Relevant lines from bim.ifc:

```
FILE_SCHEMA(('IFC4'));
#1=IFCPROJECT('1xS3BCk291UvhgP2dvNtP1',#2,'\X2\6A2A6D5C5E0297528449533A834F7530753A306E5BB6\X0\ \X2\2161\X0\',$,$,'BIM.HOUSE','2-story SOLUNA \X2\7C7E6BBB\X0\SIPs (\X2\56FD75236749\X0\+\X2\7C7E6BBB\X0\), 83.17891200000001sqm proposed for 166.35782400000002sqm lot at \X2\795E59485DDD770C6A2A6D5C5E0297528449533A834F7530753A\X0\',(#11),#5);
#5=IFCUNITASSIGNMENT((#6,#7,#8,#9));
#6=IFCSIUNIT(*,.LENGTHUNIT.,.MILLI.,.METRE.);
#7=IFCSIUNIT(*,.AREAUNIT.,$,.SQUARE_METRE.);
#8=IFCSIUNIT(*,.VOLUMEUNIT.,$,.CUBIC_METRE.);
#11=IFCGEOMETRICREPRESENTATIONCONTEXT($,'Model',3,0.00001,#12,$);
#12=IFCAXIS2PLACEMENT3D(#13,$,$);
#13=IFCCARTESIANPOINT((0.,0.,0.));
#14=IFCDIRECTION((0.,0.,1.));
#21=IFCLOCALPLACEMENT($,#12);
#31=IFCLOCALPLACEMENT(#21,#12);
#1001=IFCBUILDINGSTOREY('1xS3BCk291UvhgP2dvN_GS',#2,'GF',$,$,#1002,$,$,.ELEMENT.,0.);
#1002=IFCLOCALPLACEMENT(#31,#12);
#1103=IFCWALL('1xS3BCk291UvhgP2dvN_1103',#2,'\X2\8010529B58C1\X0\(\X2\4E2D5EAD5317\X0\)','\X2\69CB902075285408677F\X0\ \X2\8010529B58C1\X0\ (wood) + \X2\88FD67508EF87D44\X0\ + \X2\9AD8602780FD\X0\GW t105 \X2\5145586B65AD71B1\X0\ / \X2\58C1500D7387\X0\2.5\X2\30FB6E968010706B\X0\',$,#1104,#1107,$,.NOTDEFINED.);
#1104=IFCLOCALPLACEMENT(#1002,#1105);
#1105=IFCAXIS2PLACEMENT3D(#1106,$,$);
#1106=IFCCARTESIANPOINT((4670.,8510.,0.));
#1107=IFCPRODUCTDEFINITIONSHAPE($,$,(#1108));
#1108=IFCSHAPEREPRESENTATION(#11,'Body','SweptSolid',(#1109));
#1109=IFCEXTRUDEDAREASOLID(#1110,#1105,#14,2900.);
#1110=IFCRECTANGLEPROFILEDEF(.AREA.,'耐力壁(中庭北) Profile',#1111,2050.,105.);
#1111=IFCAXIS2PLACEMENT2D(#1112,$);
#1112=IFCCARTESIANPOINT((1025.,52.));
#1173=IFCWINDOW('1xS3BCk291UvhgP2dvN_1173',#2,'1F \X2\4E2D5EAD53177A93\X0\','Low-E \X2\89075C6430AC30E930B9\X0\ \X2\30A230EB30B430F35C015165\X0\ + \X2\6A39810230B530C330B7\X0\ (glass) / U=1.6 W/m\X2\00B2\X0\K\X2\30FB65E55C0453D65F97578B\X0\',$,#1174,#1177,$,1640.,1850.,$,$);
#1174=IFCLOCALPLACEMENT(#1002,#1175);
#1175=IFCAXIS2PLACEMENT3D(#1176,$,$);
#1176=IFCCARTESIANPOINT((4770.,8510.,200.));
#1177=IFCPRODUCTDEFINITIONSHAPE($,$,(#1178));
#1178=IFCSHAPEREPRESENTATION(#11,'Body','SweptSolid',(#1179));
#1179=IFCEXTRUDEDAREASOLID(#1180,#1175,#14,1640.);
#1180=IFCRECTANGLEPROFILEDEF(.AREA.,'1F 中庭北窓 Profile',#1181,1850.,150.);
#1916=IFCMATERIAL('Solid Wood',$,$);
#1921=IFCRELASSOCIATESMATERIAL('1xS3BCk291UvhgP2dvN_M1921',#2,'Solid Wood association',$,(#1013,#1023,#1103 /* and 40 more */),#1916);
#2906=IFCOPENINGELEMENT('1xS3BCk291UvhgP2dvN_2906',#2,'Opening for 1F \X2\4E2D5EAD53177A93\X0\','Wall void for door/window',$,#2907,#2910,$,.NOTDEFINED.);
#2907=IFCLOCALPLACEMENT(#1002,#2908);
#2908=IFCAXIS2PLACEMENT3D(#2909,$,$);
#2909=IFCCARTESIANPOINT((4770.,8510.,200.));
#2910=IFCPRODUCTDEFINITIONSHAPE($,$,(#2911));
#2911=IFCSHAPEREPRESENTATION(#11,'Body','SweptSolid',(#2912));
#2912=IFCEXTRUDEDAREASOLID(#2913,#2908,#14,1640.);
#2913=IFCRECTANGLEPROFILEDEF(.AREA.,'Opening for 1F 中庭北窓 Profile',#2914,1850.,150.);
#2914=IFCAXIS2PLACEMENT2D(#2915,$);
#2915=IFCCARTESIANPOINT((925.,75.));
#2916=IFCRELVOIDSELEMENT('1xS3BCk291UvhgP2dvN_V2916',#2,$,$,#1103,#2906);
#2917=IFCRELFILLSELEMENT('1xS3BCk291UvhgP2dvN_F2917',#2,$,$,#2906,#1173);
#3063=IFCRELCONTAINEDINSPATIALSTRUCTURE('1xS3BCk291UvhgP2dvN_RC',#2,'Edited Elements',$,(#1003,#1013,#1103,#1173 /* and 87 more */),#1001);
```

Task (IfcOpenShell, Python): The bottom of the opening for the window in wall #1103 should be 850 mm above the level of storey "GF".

```python
import numpy as np
import ifcopenshell
import ifcopenshell.api.geometry
import ifcopenshell.geom
import ifcopenshell.util.element
import ifcopenshell.util.placement
import ifcopenshell.util.shape
import ifcopenshell.util.unit

model = ifcopenshell.open("bim.ifc")
unit_scale = ifcopenshell.util.unit.calculate_unit_scale(model)

window = model.by_id(1173)
opening = window.FillsVoids[0].RelatingOpeningElement
storey = ifcopenshell.util.element.get_container(window, ifc_class="IfcBuildingStorey")
level = ifcopenshell.util.placement.get_local_placement(storey.ObjectPlacement)[2, 3]

# The opening's origin need not be at the sill, so measure its lowest point.
shape = ifcopenshell.geom.create_shape(ifcopenshell.geom.settings(), opening)
bottom = ifcopenshell.util.shape.get_shape_bottom_elevation(shape, shape.geometry) / unit_scale
dz = level + 0.85 / unit_scale - bottom

shift = np.array([0.0, 0.0, dz])
# The window is not placed relative to its opening, so move both.
for product in (opening, window):
    matrix = ifcopenshell.util.placement.get_local_placement(product.ObjectPlacement)
    matrix[:3, 3] += shift
    ifcopenshell.api.geometry.edit_object_placement(model, product=product, matrix=matrix, is_si=False)

print(f"moved by {dz * unit_scale:+.3f} m")

model.write("bim_rev.ifc")
```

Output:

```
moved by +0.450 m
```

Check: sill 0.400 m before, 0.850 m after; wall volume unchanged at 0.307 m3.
